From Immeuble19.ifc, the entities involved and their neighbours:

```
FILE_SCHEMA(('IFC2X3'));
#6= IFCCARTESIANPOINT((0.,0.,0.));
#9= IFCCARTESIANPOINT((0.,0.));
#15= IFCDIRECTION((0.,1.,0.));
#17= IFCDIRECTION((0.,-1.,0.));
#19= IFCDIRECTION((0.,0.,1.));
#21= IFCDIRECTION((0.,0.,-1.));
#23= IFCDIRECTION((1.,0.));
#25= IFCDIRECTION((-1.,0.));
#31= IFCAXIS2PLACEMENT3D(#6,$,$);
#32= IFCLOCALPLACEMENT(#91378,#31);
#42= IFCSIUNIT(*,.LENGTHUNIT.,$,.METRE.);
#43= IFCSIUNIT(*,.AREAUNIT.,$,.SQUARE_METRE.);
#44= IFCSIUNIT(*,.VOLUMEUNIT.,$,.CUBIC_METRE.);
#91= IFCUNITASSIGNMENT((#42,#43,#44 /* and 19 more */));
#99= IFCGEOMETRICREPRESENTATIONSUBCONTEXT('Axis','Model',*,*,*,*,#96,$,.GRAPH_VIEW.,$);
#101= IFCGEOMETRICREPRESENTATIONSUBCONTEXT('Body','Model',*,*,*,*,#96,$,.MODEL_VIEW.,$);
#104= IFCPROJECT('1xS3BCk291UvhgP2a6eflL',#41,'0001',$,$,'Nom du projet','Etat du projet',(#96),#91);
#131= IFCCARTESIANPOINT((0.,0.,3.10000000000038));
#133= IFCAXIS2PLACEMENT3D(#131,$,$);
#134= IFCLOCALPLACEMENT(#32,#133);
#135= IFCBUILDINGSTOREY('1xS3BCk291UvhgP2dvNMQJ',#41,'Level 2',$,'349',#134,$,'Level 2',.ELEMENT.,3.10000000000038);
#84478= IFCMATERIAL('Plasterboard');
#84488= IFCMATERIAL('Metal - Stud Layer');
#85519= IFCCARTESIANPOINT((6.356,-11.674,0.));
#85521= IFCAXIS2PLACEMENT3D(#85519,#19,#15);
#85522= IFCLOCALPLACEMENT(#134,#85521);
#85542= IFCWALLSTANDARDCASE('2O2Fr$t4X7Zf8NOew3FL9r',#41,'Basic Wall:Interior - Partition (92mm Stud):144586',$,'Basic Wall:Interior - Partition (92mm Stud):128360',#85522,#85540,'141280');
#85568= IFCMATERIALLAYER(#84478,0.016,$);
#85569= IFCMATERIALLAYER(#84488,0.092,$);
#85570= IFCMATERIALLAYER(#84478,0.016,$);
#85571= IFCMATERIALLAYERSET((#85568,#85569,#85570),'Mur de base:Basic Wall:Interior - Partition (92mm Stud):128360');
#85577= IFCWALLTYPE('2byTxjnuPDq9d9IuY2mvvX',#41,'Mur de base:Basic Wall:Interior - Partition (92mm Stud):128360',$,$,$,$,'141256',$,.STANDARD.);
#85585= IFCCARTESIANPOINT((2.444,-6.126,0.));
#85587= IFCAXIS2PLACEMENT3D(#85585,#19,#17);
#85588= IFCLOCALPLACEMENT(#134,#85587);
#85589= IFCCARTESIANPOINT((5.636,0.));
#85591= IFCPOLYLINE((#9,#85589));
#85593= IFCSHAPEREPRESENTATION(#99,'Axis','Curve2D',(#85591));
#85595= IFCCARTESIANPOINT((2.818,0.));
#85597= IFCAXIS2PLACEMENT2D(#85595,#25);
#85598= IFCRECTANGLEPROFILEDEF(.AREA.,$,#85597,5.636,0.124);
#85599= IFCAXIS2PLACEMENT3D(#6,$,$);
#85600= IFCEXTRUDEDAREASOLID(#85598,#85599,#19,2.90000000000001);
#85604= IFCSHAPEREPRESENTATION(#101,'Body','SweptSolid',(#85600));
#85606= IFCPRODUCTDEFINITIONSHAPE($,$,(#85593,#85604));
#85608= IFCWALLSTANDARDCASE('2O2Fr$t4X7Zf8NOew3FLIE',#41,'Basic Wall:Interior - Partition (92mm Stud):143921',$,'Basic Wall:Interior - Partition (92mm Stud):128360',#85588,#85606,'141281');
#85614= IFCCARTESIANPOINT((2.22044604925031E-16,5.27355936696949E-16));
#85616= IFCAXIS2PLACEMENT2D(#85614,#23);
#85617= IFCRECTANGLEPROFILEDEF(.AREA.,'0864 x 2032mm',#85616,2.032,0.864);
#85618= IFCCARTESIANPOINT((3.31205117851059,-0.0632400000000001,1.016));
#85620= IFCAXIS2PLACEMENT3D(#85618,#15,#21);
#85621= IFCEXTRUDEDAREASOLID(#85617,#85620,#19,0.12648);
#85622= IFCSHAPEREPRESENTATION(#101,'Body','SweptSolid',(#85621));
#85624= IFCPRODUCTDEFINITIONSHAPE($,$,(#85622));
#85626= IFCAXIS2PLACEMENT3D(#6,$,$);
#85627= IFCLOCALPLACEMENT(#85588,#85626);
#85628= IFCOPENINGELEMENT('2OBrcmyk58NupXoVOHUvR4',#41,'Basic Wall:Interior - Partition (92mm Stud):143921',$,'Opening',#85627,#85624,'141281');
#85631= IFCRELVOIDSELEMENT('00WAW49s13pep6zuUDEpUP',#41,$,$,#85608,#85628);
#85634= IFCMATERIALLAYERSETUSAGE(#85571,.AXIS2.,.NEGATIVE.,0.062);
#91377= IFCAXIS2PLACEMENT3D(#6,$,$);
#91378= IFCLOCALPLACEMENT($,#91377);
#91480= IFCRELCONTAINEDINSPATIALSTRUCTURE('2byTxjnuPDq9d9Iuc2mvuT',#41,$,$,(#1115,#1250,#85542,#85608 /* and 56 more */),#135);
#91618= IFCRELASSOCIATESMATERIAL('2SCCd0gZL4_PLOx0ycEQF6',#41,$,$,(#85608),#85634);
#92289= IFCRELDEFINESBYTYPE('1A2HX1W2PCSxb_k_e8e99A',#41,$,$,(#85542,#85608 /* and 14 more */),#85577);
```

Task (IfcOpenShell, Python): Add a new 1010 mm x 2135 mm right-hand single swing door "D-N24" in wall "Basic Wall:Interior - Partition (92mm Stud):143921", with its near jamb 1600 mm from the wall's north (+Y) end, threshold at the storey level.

```python
import numpy as np
import ifcopenshell
import ifcopenshell.api.feature
import ifcopenshell.api.geometry
import ifcopenshell.api.root
import ifcopenshell.api.spatial
import ifcopenshell.api.type
import ifcopenshell.geom
import ifcopenshell.util.element
import ifcopenshell.util.placement
import ifcopenshell.util.representation
import ifcopenshell.util.shape
import ifcopenshell.util.unit

model = ifcopenshell.open("Immeuble19.ifc")
unit_scale = ifcopenshell.util.unit.calculate_unit_scale(model)
settings = ifcopenshell.geom.settings()


def volume(element):
    """Net volume in cubic metres, openings subtracted."""
    shape = ifcopenshell.geom.create_shape(settings, element)
    return ifcopenshell.util.shape.get_volume(shape.geometry)


wall = model.by_guid("2O2Fr$t4X7Zf8NOew3FLIE")
storey = ifcopenshell.util.element.get_container(wall, ifc_class="IfcBuildingStorey")
context = ifcopenshell.util.representation.get_context(model, "Model", "Body", "MODEL_VIEW")
before = volume(wall)

width, height, from_end, sill = 1.01, 2.135, 1.6, 0.0  # metres

# The wall runs along its own X axis, and the end named is its -X end.
wall_shape = ifcopenshell.geom.create_shape(settings, wall)
x, y, z = ifcopenshell.util.shape.get_vertices(wall_shape.geometry).T
start = x.min() + from_end
face, thickness = float(y.min()), float(y.max() - y.min())
wall_matrix = ifcopenshell.util.placement.get_local_placement(wall.ObjectPlacement)
level = ifcopenshell.util.placement.get_local_placement(storey.ObjectPlacement)[2, 3]


def in_wall(x, y):
    """Placement at x, y metres in the wall's axes, at sill height."""
    matrix = wall_matrix.copy()
    matrix[:, 3] = wall_matrix @ np.array([x / unit_scale, y / unit_scale, 0.0, 1.0])
    matrix[2, 3] = level + sill / unit_scale
    return matrix


# Opening: a box that overshoots both wall faces by 50 mm.
opening = ifcopenshell.api.root.create_entity(model, ifc_class="IfcOpeningElement")
box = ifcopenshell.api.geometry.add_wall_representation(
    model, context=context, length=width, height=height, thickness=thickness + 0.1
)
ifcopenshell.api.geometry.assign_representation(model, product=opening, representation=box)
ifcopenshell.api.geometry.edit_object_placement(model, product=opening, matrix=in_wall(start, face - 0.05), is_si=False)
ifcopenshell.api.feature.add_feature(model, feature=opening, element=wall)

door = ifcopenshell.api.root.create_entity(model, ifc_class="IfcDoor", name="D-N24")
door.OverallWidth, door.OverallHeight = width / unit_scale, height / unit_scale
body = ifcopenshell.api.geometry.add_door_representation(
    model,
    context=context,
    overall_width=door.OverallWidth,
    overall_height=door.OverallHeight,
    operation_type="SINGLE_SWING_RIGHT",
    lining_properties={"LiningDepth": thickness / unit_scale, "ThresholdDepth": thickness / unit_scale},
)
ifcopenshell.api.geometry.assign_representation(model, product=door, representation=body)
ifcopenshell.api.spatial.assign_container(model, products=[door], relating_structure=storey)
fills = ifcopenshell.api.feature.add_filling(model, opening=opening, element=door)
fills.OwnerHistory = door.OwnerHistory  # required in IFC2X3

# IFC2X3 keeps the operation on the door style.
style = ifcopenshell.api.root.create_entity(model, ifc_class="IfcDoorStyle", name="D-N24")
style.OperationType, style.ConstructionType = "SINGLE_SWING_RIGHT", "NOTDEFINED"
style.ParameterTakesPrecedence = style.Sizeable = False
ifcopenshell.api.type.assign_type(model, related_objects=[door], relating_type=style)

# The lining spans the wall, so the door starts at the wall face.
ifcopenshell.api.geometry.edit_object_placement(model, product=door, matrix=in_wall(start, face), is_si=False)

after = volume(wall)

print(f"wall volume {before:.3f} -> {after:.3f} m3")

model.write("Immeuble19_updated.ifc")
```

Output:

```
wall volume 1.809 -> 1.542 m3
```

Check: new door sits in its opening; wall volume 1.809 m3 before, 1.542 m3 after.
